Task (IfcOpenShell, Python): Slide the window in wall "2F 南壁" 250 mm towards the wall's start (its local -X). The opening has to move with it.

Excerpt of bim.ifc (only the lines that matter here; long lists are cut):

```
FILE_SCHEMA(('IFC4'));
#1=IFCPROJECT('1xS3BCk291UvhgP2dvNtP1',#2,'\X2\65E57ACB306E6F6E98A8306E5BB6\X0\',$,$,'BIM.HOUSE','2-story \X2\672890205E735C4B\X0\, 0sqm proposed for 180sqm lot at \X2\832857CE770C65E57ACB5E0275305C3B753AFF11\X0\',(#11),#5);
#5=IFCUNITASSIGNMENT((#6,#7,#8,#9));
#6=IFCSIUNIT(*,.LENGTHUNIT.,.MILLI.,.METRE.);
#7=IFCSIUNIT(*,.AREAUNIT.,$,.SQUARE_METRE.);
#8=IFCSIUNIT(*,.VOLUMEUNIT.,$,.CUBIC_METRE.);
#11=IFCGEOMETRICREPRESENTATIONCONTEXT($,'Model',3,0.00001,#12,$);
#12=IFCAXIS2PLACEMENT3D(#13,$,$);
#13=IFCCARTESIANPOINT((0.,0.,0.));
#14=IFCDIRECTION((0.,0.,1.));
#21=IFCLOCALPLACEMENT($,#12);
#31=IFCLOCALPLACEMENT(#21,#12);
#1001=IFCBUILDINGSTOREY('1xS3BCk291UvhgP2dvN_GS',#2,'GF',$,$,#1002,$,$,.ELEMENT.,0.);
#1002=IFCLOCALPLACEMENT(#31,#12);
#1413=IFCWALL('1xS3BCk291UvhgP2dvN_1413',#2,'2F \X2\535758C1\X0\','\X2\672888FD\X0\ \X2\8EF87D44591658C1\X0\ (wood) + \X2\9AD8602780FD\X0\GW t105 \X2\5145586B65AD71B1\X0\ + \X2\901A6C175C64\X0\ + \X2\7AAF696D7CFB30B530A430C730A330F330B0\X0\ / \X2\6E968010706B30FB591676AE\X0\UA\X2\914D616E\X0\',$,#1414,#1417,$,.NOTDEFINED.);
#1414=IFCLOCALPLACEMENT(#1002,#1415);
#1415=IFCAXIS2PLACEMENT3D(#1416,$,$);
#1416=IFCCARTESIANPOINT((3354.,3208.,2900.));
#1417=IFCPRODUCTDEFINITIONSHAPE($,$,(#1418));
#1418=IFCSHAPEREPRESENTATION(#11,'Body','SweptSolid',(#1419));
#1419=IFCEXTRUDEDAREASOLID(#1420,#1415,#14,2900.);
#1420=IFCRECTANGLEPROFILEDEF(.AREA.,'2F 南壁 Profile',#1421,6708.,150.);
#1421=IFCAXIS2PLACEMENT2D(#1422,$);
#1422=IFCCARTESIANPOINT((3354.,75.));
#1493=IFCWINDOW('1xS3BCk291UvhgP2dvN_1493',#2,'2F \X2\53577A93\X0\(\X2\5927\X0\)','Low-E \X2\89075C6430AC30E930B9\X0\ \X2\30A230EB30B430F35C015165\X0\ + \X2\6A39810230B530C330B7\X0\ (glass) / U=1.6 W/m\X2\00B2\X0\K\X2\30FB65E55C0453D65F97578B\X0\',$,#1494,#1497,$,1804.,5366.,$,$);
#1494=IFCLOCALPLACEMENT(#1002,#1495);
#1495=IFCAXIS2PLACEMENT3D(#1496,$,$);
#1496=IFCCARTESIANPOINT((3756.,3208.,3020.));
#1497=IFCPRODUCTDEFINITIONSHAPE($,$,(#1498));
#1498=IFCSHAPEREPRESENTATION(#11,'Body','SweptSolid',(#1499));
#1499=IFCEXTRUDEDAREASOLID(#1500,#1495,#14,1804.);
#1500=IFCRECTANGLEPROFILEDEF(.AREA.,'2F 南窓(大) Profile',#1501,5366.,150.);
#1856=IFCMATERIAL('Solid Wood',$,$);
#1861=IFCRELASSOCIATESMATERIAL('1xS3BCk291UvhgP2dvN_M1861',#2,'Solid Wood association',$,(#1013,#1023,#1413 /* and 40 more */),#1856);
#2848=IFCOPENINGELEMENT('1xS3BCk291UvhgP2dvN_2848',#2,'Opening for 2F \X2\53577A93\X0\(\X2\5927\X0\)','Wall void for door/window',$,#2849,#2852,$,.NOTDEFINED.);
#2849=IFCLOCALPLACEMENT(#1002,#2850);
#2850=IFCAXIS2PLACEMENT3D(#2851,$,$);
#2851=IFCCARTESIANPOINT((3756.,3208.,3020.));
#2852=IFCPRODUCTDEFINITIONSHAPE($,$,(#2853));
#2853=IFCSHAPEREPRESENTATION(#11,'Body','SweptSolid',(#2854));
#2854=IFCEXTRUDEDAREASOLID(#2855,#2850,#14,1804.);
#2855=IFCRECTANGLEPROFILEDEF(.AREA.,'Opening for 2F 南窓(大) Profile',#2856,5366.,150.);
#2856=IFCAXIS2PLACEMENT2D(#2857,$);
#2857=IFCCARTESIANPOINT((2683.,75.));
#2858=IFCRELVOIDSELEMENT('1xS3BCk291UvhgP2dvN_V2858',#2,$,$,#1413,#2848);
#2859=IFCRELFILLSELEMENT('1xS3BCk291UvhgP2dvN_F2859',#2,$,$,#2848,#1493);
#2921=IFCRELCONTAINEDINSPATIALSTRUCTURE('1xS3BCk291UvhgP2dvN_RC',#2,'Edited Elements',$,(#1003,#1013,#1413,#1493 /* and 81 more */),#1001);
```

```python
import ifcopenshell
import ifcopenshell.api.geometry
import ifcopenshell.util.placement
import ifcopenshell.util.unit

model = ifcopenshell.open("bim.ifc")
unit_scale = ifcopenshell.util.unit.calculate_unit_scale(model)

window = model.by_guid("1xS3BCk291UvhgP2dvN_1493")
opening = window.FillsVoids[0].RelatingOpeningElement
wall = opening.VoidsElements[0].RelatingBuildingElement

wall_matrix = ifcopenshell.util.placement.get_local_placement(wall.ObjectPlacement)
shift = wall_matrix[:3, 0] * -0.25 / unit_scale
before = ifcopenshell.util.placement.get_local_placement(window.ObjectPlacement)[:3, 3].copy()

# The window is not placed relative to its opening, so move both.
for product in (opening, window):
    matrix = ifcopenshell.util.placement.get_local_placement(product.ObjectPlacement)
    matrix[:3, 3] += shift
    ifcopenshell.api.geometry.edit_object_placement(model, product=product, matrix=matrix, is_si=False)

after = ifcopenshell.util.placement.get_local_placement(window.ObjectPlacement)[:3, 3]
print("window moved by", (after - before).round(3) + 0.0)

model.write("bim_edited.ifc")
```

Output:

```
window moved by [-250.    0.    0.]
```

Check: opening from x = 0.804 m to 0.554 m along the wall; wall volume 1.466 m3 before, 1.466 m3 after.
